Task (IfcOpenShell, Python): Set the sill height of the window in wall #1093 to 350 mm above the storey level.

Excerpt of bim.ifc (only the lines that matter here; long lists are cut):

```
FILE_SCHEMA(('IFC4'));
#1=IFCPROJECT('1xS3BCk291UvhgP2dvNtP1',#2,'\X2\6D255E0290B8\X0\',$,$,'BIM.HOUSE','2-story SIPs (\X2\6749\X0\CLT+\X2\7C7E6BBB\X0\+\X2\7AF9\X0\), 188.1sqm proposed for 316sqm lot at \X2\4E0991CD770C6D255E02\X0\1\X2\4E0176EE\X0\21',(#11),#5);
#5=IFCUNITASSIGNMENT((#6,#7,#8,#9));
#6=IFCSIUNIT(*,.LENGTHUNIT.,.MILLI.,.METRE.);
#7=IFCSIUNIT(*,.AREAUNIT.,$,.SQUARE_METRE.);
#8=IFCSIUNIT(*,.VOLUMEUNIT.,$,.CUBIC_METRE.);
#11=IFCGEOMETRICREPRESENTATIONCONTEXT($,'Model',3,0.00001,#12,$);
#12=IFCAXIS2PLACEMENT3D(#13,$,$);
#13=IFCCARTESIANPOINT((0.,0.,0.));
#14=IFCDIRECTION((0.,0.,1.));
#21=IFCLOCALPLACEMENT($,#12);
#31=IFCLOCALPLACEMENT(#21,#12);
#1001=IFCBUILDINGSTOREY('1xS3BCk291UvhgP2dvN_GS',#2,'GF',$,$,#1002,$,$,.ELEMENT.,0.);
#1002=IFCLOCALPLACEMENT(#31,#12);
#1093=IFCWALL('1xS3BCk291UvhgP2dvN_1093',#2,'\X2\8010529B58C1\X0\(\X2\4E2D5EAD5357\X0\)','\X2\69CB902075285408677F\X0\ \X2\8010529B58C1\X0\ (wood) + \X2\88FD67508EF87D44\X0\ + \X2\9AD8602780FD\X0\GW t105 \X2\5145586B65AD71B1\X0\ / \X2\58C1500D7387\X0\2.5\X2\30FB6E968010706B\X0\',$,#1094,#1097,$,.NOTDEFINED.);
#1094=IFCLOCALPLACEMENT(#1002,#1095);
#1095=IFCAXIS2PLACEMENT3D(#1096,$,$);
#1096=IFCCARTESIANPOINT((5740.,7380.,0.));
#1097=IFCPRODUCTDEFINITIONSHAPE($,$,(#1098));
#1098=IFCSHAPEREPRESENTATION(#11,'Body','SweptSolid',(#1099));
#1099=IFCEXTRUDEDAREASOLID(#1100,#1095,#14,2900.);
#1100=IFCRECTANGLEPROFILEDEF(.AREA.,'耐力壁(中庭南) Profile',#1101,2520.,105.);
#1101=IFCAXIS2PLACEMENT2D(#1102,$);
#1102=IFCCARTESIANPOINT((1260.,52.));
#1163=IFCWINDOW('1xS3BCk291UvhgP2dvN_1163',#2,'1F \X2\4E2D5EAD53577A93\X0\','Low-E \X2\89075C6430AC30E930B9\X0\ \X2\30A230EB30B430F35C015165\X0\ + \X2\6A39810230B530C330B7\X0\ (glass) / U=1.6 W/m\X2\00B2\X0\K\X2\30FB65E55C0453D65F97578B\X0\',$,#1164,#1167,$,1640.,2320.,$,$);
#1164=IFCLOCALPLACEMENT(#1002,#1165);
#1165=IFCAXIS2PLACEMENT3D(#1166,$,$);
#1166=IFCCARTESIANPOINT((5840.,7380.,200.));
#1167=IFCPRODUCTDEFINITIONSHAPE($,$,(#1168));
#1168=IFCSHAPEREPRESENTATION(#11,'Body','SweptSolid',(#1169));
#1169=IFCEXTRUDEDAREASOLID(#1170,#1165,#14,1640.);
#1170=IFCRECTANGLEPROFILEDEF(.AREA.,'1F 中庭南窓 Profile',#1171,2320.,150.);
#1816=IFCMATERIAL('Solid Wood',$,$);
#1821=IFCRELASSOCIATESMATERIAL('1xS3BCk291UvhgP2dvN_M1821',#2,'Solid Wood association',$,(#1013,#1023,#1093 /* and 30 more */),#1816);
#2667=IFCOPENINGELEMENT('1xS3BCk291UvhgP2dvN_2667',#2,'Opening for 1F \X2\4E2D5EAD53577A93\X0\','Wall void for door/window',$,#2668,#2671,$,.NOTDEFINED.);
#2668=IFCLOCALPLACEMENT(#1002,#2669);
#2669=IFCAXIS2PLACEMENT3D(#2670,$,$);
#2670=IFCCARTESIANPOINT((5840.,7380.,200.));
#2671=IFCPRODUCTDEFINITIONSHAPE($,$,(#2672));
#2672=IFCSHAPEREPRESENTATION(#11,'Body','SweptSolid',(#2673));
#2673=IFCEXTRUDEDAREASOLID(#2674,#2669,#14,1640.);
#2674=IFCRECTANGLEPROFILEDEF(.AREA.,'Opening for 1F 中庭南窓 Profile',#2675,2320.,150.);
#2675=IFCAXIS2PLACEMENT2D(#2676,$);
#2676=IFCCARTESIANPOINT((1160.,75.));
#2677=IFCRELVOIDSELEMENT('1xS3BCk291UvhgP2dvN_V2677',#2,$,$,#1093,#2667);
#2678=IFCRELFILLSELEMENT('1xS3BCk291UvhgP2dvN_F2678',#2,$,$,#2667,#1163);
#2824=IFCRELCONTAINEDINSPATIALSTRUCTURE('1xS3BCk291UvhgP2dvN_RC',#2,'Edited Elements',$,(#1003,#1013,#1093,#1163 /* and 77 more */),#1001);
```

```python
import numpy as np
import ifcopenshell
import ifcopenshell.api.geometry
import ifcopenshell.geom
import ifcopenshell.util.element
import ifcopenshell.util.placement
import ifcopenshell.util.shape
import ifcopenshell.util.unit

model = ifcopenshell.open("bim.ifc")
unit_scale = ifcopenshell.util.unit.calculate_unit_scale(model)

window = model.by_guid("1xS3BCk291UvhgP2dvN_1163")
opening = window.FillsVoids[0].RelatingOpeningElement
storey = ifcopenshell.util.element.get_container(window, ifc_class="IfcBuildingStorey")
level = ifcopenshell.util.placement.get_local_placement(storey.ObjectPlacement)[2, 3]

# The opening's origin need not be at the sill, so measure its lowest point.
shape = ifcopenshell.geom.create_shape(ifcopenshell.geom.settings(), opening)
bottom = ifcopenshell.util.shape.get_shape_bottom_elevation(shape, shape.geometry) / unit_scale
dz = level + 350.0 - bottom

shift = np.array([0.0, 0.0, dz])
# The window is not placed relative to its opening, so move both.
for product in (opening, window):
    matrix = ifcopenshell.util.placement.get_local_placement(product.ObjectPlacement)
    matrix[:3, 3] += shift
    ifcopenshell.api.geometry.edit_object_placement(model, product=product, matrix=matrix, is_si=False)

print(f"moved by {dz * unit_scale:+.3f} m")

model.write("bim_rev.ifc")
```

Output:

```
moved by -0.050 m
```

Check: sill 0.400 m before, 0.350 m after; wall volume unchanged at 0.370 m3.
